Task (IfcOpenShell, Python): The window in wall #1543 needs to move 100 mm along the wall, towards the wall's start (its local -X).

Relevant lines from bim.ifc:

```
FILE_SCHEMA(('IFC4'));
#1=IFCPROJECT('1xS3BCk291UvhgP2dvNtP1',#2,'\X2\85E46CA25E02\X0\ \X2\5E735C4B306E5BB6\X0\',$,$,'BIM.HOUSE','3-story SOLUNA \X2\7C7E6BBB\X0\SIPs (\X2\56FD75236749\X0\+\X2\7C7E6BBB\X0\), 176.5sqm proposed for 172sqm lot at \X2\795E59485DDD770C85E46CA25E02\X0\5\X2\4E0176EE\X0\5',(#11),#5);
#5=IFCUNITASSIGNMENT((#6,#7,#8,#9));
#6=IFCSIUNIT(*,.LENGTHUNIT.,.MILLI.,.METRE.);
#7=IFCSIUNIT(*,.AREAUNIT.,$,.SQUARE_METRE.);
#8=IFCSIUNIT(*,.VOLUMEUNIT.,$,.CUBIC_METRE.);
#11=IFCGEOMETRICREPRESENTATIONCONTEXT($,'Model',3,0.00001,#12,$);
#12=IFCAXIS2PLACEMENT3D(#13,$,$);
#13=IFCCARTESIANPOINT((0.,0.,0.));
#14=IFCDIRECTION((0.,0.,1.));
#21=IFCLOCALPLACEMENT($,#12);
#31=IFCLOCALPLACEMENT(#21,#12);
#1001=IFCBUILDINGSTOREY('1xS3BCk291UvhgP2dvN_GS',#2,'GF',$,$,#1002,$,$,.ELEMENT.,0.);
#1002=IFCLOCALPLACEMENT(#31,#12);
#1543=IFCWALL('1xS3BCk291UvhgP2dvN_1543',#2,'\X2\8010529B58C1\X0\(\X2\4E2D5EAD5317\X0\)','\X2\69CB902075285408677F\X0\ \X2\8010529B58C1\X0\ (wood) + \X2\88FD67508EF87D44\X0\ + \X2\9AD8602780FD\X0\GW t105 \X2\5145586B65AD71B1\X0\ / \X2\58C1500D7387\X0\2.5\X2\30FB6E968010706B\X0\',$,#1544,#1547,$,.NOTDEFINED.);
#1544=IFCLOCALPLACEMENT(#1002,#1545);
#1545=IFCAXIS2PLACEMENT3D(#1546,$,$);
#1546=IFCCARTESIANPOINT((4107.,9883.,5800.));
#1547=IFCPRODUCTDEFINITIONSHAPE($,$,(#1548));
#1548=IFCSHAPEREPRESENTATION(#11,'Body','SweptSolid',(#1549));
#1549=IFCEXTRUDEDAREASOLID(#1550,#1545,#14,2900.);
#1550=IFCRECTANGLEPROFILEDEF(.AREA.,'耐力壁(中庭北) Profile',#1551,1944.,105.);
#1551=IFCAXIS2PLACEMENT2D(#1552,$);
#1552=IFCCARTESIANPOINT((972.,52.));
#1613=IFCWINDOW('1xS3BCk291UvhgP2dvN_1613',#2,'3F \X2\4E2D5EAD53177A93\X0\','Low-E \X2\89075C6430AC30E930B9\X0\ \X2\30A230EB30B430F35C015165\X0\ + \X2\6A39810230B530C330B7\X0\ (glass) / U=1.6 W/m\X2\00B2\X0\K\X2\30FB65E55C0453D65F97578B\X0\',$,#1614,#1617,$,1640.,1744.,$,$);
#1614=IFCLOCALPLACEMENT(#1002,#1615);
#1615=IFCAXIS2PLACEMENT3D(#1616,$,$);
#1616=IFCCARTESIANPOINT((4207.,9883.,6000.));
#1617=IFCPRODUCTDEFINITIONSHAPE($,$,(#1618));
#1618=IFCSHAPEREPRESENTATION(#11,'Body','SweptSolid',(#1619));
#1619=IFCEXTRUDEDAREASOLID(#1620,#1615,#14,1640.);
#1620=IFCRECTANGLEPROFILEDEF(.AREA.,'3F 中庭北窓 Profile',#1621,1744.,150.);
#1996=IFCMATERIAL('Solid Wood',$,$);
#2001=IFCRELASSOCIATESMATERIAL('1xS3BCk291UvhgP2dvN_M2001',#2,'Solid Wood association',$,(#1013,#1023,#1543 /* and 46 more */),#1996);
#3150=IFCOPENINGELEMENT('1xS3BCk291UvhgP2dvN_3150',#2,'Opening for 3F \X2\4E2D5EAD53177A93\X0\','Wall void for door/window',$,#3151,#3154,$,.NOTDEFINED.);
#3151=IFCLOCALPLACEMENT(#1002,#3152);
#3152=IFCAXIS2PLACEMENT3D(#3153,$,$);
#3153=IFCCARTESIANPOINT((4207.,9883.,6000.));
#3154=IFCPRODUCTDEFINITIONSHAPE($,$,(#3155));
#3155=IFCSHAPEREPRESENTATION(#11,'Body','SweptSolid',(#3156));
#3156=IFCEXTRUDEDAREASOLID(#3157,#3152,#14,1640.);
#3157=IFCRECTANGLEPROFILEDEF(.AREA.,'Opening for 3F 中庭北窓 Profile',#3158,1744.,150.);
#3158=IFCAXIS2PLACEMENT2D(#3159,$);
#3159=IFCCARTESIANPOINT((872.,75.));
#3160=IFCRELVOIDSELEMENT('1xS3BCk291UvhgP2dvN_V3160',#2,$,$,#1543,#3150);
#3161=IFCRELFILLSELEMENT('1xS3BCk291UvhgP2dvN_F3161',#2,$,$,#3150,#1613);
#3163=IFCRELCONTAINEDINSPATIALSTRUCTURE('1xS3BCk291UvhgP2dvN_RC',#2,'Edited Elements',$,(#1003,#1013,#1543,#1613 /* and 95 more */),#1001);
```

```python
import ifcopenshell
import ifcopenshell.api.geometry
import ifcopenshell.util.placement
import ifcopenshell.util.unit

model = ifcopenshell.open("bim.ifc")
unit_scale = ifcopenshell.util.unit.calculate_unit_scale(model)

window = model.by_id(1613)
opening = window.FillsVoids[0].RelatingOpeningElement
wall = opening.VoidsElements[0].RelatingBuildingElement

wall_matrix = ifcopenshell.util.placement.get_local_placement(wall.ObjectPlacement)
shift = wall_matrix[:3, 0] * -0.1 / unit_scale
before = ifcopenshell.util.placement.get_local_placement(window.ObjectPlacement)[:3, 3].copy()

# The window is not placed relative to its opening, so move both.
for product in (opening, window):
    matrix = ifcopenshell.util.placement.get_local_placement(product.ObjectPlacement)
    matrix[:3, 3] += shift
    ifcopenshell.api.geometry.edit_object_placement(model, product=product, matrix=matrix, is_si=False)

after = ifcopenshell.util.placement.get_local_placement(window.ObjectPlacement)[:3, 3]
print("window moved by", (after - before).round(3) + 0.0)

model.write("bim_edited.ifc")
```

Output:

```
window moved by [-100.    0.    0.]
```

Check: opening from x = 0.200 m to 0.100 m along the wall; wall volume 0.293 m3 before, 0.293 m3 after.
